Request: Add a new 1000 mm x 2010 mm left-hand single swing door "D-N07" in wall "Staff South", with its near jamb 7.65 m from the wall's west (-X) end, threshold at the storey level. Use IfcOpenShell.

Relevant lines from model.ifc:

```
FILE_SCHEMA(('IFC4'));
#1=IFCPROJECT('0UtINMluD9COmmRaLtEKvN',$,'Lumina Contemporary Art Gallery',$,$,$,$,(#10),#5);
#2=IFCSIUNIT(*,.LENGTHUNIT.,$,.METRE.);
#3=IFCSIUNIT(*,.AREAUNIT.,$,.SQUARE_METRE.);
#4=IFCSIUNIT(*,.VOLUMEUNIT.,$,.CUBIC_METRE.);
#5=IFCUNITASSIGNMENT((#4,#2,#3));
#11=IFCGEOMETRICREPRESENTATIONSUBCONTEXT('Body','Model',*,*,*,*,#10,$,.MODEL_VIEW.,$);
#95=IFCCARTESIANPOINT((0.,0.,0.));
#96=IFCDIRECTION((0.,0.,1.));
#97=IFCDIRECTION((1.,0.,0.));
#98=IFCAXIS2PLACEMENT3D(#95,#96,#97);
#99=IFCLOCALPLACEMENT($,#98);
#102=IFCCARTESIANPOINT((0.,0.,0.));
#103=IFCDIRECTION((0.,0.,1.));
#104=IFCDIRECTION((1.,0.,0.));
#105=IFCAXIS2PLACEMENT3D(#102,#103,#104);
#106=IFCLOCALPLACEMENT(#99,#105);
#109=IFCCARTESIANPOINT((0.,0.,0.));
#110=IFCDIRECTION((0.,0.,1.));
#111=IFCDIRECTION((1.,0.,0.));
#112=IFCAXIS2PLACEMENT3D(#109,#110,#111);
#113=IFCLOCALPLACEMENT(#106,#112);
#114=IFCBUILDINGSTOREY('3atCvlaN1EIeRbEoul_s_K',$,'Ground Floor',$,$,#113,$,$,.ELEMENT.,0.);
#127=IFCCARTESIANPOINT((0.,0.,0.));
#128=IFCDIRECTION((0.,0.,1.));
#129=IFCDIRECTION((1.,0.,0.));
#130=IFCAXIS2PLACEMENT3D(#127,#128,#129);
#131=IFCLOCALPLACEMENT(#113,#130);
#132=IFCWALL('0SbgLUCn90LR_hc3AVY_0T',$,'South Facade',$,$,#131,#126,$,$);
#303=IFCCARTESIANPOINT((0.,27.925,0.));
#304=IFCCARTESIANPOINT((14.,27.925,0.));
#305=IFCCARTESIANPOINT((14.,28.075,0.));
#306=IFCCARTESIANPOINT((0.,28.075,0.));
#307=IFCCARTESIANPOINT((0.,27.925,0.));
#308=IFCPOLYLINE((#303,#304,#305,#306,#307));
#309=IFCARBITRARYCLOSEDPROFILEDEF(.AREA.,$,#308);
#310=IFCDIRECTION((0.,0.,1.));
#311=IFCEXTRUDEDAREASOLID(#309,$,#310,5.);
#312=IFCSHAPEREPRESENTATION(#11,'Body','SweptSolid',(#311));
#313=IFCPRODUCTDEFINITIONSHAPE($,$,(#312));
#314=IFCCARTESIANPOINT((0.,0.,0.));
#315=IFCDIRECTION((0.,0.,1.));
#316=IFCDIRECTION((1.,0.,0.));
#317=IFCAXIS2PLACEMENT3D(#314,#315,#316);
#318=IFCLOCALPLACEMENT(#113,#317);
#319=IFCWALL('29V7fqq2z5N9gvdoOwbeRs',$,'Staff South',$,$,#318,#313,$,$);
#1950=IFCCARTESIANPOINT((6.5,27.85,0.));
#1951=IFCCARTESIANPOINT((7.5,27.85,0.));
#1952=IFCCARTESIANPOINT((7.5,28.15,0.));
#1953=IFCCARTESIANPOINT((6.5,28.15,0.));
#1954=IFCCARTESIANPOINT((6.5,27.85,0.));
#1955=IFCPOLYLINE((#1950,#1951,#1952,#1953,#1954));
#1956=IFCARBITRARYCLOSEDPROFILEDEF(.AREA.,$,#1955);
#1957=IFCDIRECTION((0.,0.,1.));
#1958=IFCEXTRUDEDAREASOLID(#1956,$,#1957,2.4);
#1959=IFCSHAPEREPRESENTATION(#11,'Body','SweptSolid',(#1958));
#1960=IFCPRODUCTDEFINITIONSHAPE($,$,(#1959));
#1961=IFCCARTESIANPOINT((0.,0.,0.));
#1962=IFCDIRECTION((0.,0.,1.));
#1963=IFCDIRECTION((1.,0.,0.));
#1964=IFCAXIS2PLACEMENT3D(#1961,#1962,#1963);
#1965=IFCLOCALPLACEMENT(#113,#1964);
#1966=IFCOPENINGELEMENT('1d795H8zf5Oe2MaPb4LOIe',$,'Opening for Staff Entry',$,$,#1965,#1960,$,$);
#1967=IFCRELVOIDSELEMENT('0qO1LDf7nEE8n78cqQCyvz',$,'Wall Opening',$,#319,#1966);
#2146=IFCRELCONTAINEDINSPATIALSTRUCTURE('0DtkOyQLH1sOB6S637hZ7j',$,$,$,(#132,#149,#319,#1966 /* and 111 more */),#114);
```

```python
import numpy as np
import ifcopenshell
import ifcopenshell.api.feature
import ifcopenshell.api.geometry
import ifcopenshell.api.root
import ifcopenshell.api.spatial
import ifcopenshell.geom
import ifcopenshell.util.element
import ifcopenshell.util.placement
import ifcopenshell.util.representation
import ifcopenshell.util.shape
import ifcopenshell.util.unit

model = ifcopenshell.open("model.ifc")
unit_scale = ifcopenshell.util.unit.calculate_unit_scale(model)
settings = ifcopenshell.geom.settings()


def volume(element):
    """Net volume in cubic metres, openings subtracted."""
    shape = ifcopenshell.geom.create_shape(settings, element)
    return ifcopenshell.util.shape.get_volume(shape.geometry)


wall = model.by_guid("29V7fqq2z5N9gvdoOwbeRs")
storey = ifcopenshell.util.element.get_container(wall, ifc_class="IfcBuildingStorey")
context = ifcopenshell.util.representation.get_context(model, "Model", "Body", "MODEL_VIEW")
before = volume(wall)

width, height, from_end, sill = 1, 2.01, 7.65, 0.0  # metres

# The wall runs along its own X axis, and the end named is its -X end.
wall_shape = ifcopenshell.geom.create_shape(settings, wall)
x, y, z = ifcopenshell.util.shape.get_vertices(wall_shape.geometry).T
start = x.min() + from_end
face, thickness = float(y.min()), float(y.max() - y.min())
wall_matrix = ifcopenshell.util.placement.get_local_placement(wall.ObjectPlacement)
level = ifcopenshell.util.placement.get_local_placement(storey.ObjectPlacement)[2, 3]


def in_wall(x, y):
    """Placement at x, y metres in the wall's axes, at sill height."""
    matrix = wall_matrix.copy()
    matrix[:, 3] = wall_matrix @ np.array([x / unit_scale, y / unit_scale, 0.0, 1.0])
    matrix[2, 3] = level + sill / unit_scale
    return matrix


# Opening: a box that overshoots both wall faces by 50 mm.
opening = ifcopenshell.api.root.create_entity(model, ifc_class="IfcOpeningElement", predefined_type="OPENING")
box = ifcopenshell.api.geometry.add_wall_representation(
    model, context=context, length=width, height=height, thickness=thickness + 0.1
)
ifcopenshell.api.geometry.assign_representation(model, product=opening, representation=box)
ifcopenshell.api.geometry.edit_object_placement(model, product=opening, matrix=in_wall(start, face - 0.05), is_si=False)
ifcopenshell.api.feature.add_feature(model, feature=opening, element=wall)

door = ifcopenshell.api.root.create_entity(model, ifc_class="IfcDoor", name="D-N07", predefined_type="DOOR")
door.OverallWidth, door.OverallHeight = width / unit_scale, height / unit_scale
door.OperationType = "SINGLE_SWING_LEFT"
body = ifcopenshell.api.geometry.add_door_representation(
    model,
    context=context,
    overall_width=door.OverallWidth,
    overall_height=door.OverallHeight,
    operation_type="SINGLE_SWING_LEFT",
    lining_properties={"LiningDepth": thickness / unit_scale, "ThresholdDepth": thickness / unit_scale},
)
ifcopenshell.api.geometry.assign_representation(model, product=door, representation=body)
ifcopenshell.api.spatial.assign_container(model, products=[door], relating_structure=storey)
ifcopenshell.api.feature.add_filling(model, opening=opening, element=door)

# The lining spans the wall, so the door starts at the wall face.
ifcopenshell.api.geometry.edit_object_placement(model, product=door, matrix=in_wall(start, face), is_si=False)

after = volume(wall)

print(f"wall volume {before:.3f} -> {after:.3f} m3")

model.write("model_edited.ifc")
```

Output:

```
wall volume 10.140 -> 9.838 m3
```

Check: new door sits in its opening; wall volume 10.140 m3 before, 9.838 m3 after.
